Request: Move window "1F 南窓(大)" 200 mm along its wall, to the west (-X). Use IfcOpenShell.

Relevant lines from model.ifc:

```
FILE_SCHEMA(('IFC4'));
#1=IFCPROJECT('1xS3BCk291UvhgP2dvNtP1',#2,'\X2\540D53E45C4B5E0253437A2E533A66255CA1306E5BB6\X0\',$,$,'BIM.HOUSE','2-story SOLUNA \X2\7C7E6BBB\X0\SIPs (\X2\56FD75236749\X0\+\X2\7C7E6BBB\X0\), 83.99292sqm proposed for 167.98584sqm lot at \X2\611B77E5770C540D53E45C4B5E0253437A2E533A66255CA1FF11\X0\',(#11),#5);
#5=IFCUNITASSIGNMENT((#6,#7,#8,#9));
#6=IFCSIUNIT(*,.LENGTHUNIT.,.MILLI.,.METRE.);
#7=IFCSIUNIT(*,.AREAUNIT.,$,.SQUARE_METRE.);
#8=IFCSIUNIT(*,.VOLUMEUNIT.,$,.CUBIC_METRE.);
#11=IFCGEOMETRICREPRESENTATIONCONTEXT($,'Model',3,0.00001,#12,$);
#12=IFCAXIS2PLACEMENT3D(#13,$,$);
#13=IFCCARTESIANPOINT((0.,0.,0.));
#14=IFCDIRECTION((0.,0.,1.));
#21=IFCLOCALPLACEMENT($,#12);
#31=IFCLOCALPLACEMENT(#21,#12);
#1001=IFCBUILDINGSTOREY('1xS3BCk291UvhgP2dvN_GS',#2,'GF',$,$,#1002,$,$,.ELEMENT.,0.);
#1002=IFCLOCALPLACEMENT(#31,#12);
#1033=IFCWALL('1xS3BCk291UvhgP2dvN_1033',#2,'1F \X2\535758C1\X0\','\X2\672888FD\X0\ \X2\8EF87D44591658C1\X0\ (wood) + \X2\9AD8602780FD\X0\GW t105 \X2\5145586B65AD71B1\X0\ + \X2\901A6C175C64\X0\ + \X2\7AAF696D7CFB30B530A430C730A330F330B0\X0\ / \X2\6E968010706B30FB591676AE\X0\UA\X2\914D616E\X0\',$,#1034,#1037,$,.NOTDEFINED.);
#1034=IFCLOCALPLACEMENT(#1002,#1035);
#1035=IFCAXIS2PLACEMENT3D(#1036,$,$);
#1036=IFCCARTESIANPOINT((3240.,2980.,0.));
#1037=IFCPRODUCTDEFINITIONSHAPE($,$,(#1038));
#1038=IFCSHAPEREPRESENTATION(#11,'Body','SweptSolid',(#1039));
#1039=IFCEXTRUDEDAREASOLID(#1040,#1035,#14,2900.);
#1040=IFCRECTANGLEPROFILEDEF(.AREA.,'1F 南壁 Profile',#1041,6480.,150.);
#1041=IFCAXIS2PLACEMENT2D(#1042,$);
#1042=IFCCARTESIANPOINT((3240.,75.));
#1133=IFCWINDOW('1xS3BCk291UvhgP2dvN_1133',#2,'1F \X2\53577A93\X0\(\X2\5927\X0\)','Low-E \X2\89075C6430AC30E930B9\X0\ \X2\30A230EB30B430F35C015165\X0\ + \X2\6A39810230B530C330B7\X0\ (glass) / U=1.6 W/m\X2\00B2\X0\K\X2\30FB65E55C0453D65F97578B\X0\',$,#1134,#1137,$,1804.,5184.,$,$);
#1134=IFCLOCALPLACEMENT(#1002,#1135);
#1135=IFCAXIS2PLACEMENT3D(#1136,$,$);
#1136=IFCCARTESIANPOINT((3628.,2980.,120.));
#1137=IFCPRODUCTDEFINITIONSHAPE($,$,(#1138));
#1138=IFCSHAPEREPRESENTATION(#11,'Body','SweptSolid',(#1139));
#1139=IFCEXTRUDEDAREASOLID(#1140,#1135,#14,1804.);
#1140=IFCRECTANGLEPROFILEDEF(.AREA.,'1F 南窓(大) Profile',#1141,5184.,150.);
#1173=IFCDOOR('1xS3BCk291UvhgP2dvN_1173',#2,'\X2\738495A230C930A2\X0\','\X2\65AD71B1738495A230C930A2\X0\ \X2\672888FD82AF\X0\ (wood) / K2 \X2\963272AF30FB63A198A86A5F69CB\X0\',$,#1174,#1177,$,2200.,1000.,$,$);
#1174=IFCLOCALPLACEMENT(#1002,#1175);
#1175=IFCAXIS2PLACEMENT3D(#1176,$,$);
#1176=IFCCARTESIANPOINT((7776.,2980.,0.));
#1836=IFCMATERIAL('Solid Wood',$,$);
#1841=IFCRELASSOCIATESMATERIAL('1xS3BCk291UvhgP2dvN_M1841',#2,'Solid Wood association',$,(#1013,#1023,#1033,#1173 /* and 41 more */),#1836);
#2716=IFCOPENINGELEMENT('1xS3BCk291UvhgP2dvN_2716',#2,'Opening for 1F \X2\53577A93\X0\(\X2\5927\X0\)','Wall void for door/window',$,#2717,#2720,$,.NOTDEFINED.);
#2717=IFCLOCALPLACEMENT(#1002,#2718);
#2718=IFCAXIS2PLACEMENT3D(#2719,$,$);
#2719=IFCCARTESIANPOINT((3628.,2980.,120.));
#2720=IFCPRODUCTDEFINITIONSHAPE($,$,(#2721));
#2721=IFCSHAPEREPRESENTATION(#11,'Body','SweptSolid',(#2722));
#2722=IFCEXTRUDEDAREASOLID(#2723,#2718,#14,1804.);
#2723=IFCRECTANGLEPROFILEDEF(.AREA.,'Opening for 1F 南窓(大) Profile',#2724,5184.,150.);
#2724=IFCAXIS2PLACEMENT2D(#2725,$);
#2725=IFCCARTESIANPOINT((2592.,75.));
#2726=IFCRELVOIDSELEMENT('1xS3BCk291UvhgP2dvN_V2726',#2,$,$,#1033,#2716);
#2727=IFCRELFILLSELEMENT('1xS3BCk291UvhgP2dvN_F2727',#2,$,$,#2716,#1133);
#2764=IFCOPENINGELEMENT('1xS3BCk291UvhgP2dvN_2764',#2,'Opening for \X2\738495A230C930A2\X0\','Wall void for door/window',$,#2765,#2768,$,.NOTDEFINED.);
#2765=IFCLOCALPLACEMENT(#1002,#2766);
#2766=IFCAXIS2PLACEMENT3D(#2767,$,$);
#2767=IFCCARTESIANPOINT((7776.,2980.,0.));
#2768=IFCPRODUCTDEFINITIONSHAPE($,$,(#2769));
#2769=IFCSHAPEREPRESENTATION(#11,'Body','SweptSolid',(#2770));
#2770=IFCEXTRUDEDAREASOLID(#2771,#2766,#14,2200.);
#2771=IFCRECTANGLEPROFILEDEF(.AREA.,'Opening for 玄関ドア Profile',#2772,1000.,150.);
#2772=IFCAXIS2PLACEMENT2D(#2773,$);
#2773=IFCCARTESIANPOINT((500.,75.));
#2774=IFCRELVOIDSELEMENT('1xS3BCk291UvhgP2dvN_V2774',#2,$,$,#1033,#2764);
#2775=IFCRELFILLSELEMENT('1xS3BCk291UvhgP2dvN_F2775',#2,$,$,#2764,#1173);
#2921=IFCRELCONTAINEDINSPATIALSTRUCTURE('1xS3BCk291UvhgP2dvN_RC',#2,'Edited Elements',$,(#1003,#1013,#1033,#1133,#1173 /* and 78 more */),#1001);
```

```python
import ifcopenshell
import ifcopenshell.api.geometry
import ifcopenshell.util.placement

model = ifcopenshell.open("model.ifc")

window = model.by_id(1133)
opening = window.FillsVoids[0].RelatingOpeningElement
wall = opening.VoidsElements[0].RelatingBuildingElement

wall_matrix = ifcopenshell.util.placement.get_local_placement(wall.ObjectPlacement)
shift = wall_matrix[:3, 0] * -200.0
before = ifcopenshell.util.placement.get_local_placement(window.ObjectPlacement)[:3, 3].copy()

# The window is not placed relative to its opening, so move both.
for product in (opening, window):
    matrix = ifcopenshell.util.placement.get_local_placement(product.ObjectPlacement)
    matrix[:3, 3] += shift
    ifcopenshell.api.geometry.edit_object_placement(model, product=product, matrix=matrix, is_si=False)

after = ifcopenshell.util.placement.get_local_placement(window.ObjectPlacement)[:3, 3]
print("window moved by", (after - before).round(3) + 0.0)

model.write("model_v2.ifc")
```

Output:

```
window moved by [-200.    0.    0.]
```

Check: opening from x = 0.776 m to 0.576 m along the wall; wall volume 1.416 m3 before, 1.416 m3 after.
